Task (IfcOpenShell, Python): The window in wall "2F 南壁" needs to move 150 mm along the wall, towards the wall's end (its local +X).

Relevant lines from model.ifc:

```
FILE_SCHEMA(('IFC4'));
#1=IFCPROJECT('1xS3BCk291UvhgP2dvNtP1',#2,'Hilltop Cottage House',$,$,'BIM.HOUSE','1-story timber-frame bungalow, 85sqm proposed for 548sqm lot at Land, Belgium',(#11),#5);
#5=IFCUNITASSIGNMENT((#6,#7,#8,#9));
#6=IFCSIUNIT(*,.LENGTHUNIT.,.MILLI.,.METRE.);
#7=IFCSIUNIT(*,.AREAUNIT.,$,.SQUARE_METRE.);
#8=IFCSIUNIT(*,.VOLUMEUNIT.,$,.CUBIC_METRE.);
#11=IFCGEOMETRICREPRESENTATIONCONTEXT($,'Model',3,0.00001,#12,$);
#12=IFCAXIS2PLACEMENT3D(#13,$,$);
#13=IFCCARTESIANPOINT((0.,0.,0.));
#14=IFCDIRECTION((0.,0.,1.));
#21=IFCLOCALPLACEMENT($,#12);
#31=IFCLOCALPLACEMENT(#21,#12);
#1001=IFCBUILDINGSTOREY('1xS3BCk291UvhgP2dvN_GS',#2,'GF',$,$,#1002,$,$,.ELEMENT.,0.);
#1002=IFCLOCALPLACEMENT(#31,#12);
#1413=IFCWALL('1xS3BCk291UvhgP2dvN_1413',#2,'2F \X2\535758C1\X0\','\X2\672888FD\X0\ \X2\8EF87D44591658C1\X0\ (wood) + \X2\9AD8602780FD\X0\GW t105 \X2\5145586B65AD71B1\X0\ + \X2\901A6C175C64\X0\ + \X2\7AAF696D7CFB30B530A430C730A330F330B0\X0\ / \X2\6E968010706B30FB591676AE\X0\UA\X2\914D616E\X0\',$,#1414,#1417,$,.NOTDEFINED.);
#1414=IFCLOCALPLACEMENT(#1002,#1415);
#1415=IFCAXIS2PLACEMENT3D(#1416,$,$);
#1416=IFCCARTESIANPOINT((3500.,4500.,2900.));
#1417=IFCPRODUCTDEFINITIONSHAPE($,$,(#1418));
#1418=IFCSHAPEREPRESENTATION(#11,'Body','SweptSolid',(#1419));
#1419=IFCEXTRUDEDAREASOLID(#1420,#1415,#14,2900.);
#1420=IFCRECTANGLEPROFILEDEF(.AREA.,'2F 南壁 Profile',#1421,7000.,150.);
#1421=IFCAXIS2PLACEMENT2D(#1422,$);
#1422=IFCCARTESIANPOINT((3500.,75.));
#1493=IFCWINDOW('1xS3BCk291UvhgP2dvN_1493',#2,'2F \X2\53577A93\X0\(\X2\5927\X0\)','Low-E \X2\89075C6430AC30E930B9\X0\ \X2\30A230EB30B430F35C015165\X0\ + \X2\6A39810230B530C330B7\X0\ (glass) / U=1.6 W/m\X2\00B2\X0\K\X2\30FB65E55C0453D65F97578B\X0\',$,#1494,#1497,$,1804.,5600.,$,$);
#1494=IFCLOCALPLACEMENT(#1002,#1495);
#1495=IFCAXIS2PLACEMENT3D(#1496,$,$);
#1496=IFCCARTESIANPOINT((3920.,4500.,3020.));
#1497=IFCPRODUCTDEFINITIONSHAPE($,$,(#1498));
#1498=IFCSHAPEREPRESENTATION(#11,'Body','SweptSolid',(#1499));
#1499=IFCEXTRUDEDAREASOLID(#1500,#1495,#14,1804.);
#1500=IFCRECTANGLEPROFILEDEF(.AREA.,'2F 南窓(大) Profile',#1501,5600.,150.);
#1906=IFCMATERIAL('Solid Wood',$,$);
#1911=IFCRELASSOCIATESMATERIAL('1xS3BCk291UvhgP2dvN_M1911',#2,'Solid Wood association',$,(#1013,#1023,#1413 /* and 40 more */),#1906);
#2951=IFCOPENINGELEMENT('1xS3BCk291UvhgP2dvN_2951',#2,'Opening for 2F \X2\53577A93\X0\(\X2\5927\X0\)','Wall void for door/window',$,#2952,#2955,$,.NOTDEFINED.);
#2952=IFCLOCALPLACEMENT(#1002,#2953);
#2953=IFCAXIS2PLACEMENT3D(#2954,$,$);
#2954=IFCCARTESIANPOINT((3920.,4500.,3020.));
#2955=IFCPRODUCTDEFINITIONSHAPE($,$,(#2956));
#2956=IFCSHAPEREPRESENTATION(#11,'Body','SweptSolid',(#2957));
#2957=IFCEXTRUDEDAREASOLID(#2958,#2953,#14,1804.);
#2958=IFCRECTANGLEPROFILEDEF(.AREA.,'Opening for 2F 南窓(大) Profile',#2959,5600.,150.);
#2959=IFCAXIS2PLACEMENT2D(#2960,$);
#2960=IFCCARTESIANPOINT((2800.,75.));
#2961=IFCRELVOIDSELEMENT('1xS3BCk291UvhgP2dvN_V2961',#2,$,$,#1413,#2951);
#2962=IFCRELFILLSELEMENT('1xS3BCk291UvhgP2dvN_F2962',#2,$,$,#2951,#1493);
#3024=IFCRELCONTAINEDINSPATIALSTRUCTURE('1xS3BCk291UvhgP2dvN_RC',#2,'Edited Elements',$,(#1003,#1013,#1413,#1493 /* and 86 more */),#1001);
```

```python
import ifcopenshell
import ifcopenshell.api.geometry
import ifcopenshell.util.placement
import ifcopenshell.util.unit

model = ifcopenshell.open("model.ifc")
unit_scale = ifcopenshell.util.unit.calculate_unit_scale(model)

window = model.by_id(1493)
opening = window.FillsVoids[0].RelatingOpeningElement
wall = opening.VoidsElements[0].RelatingBuildingElement

wall_matrix = ifcopenshell.util.placement.get_local_placement(wall.ObjectPlacement)
shift = wall_matrix[:3, 0] * 0.15 / unit_scale
before = ifcopenshell.util.placement.get_local_placement(window.ObjectPlacement)[:3, 3].copy()

# The window is not placed relative to its opening, so move both.
for product in (opening, window):
    matrix = ifcopenshell.util.placement.get_local_placement(product.ObjectPlacement)
    matrix[:3, 3] += shift
    ifcopenshell.api.geometry.edit_object_placement(model, product=product, matrix=matrix, is_si=False)

after = ifcopenshell.util.placement.get_local_placement(window.ObjectPlacement)[:3, 3]
print("window moved by", (after - before).round(3) + 0.0)

model.write("model_updated.ifc")
```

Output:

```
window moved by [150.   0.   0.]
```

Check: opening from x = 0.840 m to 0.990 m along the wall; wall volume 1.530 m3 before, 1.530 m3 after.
